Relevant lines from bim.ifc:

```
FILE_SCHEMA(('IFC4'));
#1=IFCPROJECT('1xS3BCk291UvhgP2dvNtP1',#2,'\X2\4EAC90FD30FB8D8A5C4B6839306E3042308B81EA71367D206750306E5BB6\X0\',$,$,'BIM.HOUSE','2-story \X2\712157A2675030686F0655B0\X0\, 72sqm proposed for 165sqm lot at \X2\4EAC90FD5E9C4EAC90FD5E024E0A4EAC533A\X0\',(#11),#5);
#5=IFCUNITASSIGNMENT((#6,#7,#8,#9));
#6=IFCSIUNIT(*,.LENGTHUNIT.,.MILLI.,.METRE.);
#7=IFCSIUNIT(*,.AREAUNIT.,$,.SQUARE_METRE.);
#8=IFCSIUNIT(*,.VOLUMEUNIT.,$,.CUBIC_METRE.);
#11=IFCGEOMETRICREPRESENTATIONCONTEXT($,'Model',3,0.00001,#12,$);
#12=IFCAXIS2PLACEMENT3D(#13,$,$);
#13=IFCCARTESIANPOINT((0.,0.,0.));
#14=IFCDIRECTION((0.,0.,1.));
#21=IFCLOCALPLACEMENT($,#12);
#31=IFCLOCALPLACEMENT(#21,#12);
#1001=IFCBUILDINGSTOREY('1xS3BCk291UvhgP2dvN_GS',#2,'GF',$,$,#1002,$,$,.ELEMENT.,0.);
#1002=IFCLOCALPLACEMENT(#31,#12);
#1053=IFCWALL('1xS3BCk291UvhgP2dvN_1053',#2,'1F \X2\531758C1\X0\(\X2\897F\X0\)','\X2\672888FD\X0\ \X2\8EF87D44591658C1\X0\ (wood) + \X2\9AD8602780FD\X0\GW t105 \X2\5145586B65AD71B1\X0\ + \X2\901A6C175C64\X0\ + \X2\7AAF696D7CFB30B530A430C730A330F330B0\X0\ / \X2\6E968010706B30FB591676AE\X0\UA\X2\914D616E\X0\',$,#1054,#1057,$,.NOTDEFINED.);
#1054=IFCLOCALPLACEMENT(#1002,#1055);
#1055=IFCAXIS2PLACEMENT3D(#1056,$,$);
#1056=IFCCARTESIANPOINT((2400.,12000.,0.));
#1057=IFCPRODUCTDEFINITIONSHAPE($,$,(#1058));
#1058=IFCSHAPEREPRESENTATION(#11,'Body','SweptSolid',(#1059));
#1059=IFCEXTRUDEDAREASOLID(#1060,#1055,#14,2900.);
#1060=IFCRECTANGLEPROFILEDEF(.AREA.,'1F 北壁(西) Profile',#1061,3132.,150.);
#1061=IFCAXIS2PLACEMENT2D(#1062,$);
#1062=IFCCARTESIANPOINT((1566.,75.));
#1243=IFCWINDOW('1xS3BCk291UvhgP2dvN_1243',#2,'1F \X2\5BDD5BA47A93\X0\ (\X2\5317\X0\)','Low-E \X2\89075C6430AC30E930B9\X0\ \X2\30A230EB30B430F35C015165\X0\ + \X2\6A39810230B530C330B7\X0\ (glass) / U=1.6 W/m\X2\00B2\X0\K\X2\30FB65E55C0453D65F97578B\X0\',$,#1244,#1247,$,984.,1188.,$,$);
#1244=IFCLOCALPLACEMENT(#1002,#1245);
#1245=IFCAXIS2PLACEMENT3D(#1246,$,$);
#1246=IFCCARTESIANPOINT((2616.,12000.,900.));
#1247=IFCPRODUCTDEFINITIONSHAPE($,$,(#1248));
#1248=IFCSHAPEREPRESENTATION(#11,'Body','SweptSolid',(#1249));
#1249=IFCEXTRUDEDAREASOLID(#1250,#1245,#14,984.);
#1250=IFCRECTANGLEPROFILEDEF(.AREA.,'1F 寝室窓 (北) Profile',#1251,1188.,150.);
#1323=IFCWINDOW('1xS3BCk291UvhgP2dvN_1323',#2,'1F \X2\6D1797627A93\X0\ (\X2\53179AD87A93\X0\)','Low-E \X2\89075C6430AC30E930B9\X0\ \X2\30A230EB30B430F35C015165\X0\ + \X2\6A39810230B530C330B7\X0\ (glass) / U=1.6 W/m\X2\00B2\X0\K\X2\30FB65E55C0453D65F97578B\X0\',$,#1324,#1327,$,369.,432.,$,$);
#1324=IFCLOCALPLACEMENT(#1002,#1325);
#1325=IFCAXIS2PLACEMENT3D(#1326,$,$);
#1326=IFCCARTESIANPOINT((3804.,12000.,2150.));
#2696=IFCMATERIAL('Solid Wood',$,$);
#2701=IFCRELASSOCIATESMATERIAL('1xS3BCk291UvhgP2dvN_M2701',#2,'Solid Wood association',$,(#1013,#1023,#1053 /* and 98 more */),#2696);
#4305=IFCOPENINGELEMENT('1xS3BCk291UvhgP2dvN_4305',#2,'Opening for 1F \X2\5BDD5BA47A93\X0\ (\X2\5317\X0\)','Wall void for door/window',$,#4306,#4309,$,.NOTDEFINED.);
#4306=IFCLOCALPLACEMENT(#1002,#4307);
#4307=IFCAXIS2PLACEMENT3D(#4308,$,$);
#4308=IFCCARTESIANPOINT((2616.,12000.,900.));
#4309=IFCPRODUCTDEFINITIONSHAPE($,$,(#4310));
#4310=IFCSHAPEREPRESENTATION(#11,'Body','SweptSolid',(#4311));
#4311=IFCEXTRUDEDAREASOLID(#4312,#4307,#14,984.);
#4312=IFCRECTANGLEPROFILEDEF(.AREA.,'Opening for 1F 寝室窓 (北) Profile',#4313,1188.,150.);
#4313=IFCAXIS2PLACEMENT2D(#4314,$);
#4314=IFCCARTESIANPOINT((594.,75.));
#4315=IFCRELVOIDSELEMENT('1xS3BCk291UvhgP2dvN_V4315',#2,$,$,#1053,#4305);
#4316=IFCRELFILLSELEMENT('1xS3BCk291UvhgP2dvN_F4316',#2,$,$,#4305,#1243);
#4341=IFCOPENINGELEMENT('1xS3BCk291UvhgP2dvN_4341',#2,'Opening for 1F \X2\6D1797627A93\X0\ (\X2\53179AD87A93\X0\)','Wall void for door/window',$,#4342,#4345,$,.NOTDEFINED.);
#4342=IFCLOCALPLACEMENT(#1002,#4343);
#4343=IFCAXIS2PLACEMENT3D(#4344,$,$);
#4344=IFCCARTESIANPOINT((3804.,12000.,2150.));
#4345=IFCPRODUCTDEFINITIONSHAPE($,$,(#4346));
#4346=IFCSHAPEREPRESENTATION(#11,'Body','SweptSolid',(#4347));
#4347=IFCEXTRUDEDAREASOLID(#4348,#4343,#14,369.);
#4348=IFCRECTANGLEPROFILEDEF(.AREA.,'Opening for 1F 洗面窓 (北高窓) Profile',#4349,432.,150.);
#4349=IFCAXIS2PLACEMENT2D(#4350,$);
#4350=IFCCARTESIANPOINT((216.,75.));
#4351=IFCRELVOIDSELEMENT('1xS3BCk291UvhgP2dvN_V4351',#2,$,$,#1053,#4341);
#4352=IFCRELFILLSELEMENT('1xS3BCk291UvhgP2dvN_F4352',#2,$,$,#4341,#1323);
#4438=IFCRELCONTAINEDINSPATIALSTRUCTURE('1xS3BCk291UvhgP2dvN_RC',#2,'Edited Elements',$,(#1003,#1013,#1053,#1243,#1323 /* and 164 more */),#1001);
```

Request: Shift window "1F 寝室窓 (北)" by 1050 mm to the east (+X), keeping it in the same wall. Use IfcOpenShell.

```python
import ifcopenshell
import ifcopenshell.api.geometry
import ifcopenshell.util.placement

model = ifcopenshell.open("bim.ifc")

window = model.by_id(1243)
opening = window.FillsVoids[0].RelatingOpeningElement
wall = opening.VoidsElements[0].RelatingBuildingElement

wall_matrix = ifcopenshell.util.placement.get_local_placement(wall.ObjectPlacement)
shift = wall_matrix[:3, 0] * 1050.0
before = ifcopenshell.util.placement.get_local_placement(window.ObjectPlacement)[:3, 3].copy()

# The window is not placed relative to its opening, so move both.
for product in (opening, window):
    matrix = ifcopenshell.util.placement.get_local_placement(product.ObjectPlacement)
    matrix[:3, 3] += shift
    ifcopenshell.api.geometry.edit_object_placement(model, product=product, matrix=matrix, is_si=False)

after = ifcopenshell.util.placement.get_local_placement(window.ObjectPlacement)[:3, 3]
print("window moved by", (after - before).round(3) + 0.0)

model.write("bim_updated.ifc")
```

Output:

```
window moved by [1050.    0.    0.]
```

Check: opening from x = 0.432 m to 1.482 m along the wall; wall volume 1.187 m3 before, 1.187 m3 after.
